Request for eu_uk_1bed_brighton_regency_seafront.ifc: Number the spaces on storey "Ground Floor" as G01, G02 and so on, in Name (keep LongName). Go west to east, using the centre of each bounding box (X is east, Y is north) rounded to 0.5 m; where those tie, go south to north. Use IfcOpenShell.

First a look at what the model holds.

```python
import ifcopenshell
import ifcopenshell.util.element
import ifcopenshell.util.placement

model = ifcopenshell.open("eu_uk_1bed_brighton_regency_seafront.ifc")
print(model.schema)
storey = next(s for s in model.by_type("IfcBuildingStorey") if s.Name == "Ground Floor")
spaces = [e for e in ifcopenshell.util.element.get_decomposition(storey) if e.is_a("IfcSpace")]
for e in sorted(spaces, key=lambda e: e.id()):
    origin = ifcopenshell.util.placement.get_local_placement(e.ObjectPlacement)[:3, 3]
    print(e.id(), e.Name, e.LongName, origin.round(2) + 0.0, sep=" | ")
```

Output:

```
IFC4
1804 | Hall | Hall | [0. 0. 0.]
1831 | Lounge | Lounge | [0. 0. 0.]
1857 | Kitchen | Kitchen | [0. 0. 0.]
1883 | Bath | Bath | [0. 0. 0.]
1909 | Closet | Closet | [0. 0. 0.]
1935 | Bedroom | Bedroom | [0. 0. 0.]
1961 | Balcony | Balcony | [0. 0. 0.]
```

```python
import ifcopenshell
import ifcopenshell.geom
import ifcopenshell.util.element
import ifcopenshell.util.shape

model = ifcopenshell.open("eu_uk_1bed_brighton_regency_seafront.ifc")
settings = ifcopenshell.geom.settings()
settings.set("use-world-coords", True)


def centre(element):
    shape = ifcopenshell.geom.create_shape(settings, element)
    return ifcopenshell.util.shape.get_bbox_centroid(shape.geometry)


storey = next(s for s in model.by_type("IfcBuildingStorey") if s.Name == "Ground Floor")
spaces = [e for e in ifcopenshell.util.element.get_decomposition(storey) if e.is_a("IfcSpace")]

# Insertion points can sit at a corner or the storey origin, so sort by the geometry (in metres).
centres = {e: centre(e) for e in spaces}
spaces.sort(key=lambda e: (round(centres[e][0] / 0.5), centres[e][1]))

for i, e in enumerate(spaces, start=1):
    number = f"G{i:02d}"
    e.Name = number
    print(e.id(), number)

model.write("eu_uk_1bed_brighton_regency_seafront-out.ifc")
```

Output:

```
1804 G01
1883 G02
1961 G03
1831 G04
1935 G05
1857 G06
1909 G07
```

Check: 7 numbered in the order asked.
